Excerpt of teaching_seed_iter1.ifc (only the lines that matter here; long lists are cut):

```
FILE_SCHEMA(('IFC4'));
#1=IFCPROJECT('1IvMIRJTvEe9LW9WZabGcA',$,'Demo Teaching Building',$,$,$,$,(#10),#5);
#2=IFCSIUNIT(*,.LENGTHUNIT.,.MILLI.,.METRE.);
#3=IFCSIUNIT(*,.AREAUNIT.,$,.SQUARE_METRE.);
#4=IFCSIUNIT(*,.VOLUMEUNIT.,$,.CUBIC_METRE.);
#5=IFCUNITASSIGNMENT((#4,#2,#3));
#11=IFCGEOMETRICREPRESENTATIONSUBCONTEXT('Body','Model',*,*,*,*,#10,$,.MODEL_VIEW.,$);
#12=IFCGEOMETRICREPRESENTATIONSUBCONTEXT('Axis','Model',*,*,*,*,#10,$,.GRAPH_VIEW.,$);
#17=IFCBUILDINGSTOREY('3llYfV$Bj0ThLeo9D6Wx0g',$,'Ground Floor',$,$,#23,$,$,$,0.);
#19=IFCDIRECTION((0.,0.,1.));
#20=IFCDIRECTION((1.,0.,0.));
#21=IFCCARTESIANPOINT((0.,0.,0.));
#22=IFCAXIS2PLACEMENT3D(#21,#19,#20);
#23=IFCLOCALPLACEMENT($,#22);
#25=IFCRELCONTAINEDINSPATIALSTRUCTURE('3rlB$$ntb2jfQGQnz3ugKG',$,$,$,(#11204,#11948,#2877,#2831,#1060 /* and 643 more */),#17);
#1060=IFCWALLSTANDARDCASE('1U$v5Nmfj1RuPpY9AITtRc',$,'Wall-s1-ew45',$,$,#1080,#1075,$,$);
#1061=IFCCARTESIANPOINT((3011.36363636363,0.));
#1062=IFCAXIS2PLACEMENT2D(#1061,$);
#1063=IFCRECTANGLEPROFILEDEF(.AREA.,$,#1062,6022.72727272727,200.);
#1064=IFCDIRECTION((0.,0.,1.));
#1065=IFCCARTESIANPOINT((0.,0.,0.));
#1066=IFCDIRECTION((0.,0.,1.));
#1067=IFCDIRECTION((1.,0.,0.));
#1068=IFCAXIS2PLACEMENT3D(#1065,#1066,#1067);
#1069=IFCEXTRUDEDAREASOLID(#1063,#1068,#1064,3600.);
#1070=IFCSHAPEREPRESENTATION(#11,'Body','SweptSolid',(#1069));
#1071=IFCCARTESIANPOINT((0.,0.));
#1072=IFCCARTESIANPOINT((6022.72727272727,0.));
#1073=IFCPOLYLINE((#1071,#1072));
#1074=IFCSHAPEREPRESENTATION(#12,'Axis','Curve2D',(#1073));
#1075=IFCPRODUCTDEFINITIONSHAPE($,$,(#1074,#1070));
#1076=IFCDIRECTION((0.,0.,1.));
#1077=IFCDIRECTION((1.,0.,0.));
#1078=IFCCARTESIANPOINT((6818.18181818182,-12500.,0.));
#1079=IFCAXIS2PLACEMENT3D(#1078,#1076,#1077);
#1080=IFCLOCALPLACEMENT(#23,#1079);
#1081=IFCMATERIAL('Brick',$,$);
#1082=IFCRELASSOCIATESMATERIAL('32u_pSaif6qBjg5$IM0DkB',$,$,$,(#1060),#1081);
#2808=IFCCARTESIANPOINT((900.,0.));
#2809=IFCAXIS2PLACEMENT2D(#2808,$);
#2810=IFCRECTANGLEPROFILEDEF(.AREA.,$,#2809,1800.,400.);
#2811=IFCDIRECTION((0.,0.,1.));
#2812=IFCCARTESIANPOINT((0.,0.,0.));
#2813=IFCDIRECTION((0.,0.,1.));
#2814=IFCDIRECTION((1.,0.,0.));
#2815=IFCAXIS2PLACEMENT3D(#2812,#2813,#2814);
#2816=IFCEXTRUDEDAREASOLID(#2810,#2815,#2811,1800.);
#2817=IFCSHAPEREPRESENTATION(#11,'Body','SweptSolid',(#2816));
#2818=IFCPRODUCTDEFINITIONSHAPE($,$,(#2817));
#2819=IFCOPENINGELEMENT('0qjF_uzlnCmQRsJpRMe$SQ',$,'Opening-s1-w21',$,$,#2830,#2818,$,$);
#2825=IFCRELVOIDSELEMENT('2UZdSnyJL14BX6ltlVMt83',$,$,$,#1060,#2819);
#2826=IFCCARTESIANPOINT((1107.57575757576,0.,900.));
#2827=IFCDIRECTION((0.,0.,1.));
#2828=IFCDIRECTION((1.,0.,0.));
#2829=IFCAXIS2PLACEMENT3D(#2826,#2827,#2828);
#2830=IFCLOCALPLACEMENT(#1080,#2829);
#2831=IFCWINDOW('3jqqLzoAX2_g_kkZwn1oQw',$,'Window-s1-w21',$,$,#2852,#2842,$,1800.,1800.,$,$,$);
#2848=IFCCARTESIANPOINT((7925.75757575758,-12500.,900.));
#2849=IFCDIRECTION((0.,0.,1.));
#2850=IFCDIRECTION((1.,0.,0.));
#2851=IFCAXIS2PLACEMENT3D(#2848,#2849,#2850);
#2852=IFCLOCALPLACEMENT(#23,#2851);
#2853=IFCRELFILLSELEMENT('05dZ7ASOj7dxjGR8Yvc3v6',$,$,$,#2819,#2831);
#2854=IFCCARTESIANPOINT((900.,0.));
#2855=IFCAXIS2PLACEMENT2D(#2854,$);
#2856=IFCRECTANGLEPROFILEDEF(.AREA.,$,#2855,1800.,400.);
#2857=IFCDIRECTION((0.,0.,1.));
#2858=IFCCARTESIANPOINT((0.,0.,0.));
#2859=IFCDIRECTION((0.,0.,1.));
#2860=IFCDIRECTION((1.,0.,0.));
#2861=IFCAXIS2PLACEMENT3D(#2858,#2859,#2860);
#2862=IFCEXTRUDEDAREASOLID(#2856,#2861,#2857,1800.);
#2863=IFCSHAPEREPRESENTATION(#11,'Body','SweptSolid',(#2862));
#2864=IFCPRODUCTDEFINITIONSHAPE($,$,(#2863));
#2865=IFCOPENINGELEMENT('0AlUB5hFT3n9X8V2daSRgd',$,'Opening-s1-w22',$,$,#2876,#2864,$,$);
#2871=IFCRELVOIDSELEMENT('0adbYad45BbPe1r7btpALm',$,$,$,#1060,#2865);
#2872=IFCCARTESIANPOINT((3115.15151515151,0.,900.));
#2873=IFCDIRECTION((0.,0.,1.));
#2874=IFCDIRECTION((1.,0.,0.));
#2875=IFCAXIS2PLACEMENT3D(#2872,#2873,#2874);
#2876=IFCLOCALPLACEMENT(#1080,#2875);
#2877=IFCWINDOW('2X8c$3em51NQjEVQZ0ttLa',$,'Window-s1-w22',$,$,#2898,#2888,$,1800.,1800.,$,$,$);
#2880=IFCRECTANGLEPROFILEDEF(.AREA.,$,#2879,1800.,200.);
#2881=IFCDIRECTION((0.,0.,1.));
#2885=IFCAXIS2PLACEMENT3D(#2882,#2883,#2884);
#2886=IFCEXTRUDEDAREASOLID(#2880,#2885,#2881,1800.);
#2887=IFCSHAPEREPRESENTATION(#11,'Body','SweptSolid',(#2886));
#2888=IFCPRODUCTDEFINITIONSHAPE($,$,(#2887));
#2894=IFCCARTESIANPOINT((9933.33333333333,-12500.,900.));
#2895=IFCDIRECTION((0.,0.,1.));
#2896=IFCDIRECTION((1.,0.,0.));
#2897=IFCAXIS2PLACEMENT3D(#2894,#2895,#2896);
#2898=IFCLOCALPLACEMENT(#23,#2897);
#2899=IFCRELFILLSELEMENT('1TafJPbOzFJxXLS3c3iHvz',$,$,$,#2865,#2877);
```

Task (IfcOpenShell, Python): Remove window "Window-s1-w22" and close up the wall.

```python
import ifcopenshell
import ifcopenshell.api.feature
import ifcopenshell.api.root
import ifcopenshell.geom
import ifcopenshell.util.shape

model = ifcopenshell.open("teaching_seed_iter1.ifc")
settings = ifcopenshell.geom.settings()


def volume(element):
    """Net volume in cubic metres, openings subtracted."""
    shape = ifcopenshell.geom.create_shape(settings, element)
    return ifcopenshell.util.shape.get_volume(shape.geometry)


window = model.by_guid("2X8c$3em51NQjEVQZ0ttLa")
opening = window.FillsVoids[0].RelatingOpeningElement
wall = opening.VoidsElements[0].RelatingBuildingElement
before = volume(wall)

ifcopenshell.api.root.remove_product(model, product=window)
ifcopenshell.api.feature.remove_feature(model, feature=opening)

after = volume(wall)

print(f"wall volume {before:.3f} -> {after:.3f} m3")

model.write("teaching_seed_iter1-out.ifc")
```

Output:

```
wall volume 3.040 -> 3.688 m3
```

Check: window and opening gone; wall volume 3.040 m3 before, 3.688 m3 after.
